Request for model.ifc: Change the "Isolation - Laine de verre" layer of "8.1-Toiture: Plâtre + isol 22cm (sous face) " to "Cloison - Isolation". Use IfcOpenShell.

First a look at what the model holds.

```python
import ifcopenshell
import ifcopenshell.util.element

model = ifcopenshell.open("model.ifc")
print(model.schema)
for layer_set in model.by_type("IfcMaterialLayerSet"):
    if layer_set.LayerSetName == "8.1-Toiture: Plâtre + isol 22cm (sous face) ":
        for layer in layer_set.MaterialLayers:
            print(layer.id(), layer.Material and layer.Material.Name, layer.LayerThickness, sep=" | ")
        print(len(ifcopenshell.util.element.get_elements_by_material(model, layer_set)), "elements and types use it")
print(sorted(m.Name for m in model.by_type("IfcMaterial") if m.Name)[:60])
```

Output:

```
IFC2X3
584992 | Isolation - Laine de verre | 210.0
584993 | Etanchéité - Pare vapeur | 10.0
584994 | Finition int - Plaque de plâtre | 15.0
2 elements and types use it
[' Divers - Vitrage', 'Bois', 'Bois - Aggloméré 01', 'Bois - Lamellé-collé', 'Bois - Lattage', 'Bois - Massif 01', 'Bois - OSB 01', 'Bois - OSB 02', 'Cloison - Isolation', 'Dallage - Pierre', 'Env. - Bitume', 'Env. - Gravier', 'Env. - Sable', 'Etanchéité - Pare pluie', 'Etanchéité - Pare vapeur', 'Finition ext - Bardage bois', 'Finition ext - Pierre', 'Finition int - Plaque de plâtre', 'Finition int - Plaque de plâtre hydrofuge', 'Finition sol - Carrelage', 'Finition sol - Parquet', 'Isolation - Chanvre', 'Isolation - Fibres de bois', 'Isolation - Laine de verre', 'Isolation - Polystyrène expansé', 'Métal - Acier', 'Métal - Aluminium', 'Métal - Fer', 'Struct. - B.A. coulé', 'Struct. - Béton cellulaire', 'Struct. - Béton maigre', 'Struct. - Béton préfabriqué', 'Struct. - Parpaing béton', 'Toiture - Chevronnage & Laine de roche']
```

```python
import ifcopenshell
import ifcopenshell.api.material

model = ifcopenshell.open("model.ifc")

layer_set = next(s for s in model.by_type("IfcMaterialLayerSet") if s.LayerSetName == "8.1-Toiture: Plâtre + isol 22cm (sous face) ")
layer = next(l for l in layer_set.MaterialLayers if l.Material and l.Material.Name == "Isolation - Laine de verre")
material = next(m for m in model.by_type("IfcMaterial") if m.Name == "Cloison - Isolation")

# Point this one layer at the other material; renaming the old one would change it everywhere.
ifcopenshell.api.material.edit_layer(model, layer=layer, attributes={}, material=material)

print([l.Material.Name if l.Material else None for l in layer_set.MaterialLayers])

model.write("model_edited.ifc")
```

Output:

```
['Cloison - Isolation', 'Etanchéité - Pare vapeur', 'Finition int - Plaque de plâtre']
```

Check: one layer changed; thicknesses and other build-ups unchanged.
